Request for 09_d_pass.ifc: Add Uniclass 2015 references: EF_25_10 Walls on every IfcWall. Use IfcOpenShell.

First a look at what the model holds.

```python
import ifcopenshell

model = ifcopenshell.open("09_d_pass.ifc")
print(model.schema)
print("classifications:", [c.Name for c in model.by_type("IfcClassification")])
for ifc_class in ("IfcDoor", "IfcRoof", "IfcStair", "IfcWall", "IfcWindow"):
    print(ifc_class, len(model.by_type(ifc_class)))
```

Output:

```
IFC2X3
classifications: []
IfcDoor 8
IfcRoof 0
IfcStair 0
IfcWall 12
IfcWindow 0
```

```python
import ifcopenshell
import ifcopenshell.api.classification

model = ifcopenshell.open("09_d_pass.ifc")

# IFC2X3 requires Source and Edition and has no link from the project to the system.
system = model.create_entity("IfcClassification", Source="NBS", Edition="2015", Name="Uniclass 2015")

codes = {
    "IfcWall": ("EF_25_10", "Walls"),
}
for ifc_class, (code, name) in codes.items():
    products = model.by_type(ifc_class)
    ifcopenshell.api.classification.add_reference(
        model, products=products, classification=system, identification=code, name=name
    )
    print(code, len(products))

model.write("09_d_pass-out.ifc")
```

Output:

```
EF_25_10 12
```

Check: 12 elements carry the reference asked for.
